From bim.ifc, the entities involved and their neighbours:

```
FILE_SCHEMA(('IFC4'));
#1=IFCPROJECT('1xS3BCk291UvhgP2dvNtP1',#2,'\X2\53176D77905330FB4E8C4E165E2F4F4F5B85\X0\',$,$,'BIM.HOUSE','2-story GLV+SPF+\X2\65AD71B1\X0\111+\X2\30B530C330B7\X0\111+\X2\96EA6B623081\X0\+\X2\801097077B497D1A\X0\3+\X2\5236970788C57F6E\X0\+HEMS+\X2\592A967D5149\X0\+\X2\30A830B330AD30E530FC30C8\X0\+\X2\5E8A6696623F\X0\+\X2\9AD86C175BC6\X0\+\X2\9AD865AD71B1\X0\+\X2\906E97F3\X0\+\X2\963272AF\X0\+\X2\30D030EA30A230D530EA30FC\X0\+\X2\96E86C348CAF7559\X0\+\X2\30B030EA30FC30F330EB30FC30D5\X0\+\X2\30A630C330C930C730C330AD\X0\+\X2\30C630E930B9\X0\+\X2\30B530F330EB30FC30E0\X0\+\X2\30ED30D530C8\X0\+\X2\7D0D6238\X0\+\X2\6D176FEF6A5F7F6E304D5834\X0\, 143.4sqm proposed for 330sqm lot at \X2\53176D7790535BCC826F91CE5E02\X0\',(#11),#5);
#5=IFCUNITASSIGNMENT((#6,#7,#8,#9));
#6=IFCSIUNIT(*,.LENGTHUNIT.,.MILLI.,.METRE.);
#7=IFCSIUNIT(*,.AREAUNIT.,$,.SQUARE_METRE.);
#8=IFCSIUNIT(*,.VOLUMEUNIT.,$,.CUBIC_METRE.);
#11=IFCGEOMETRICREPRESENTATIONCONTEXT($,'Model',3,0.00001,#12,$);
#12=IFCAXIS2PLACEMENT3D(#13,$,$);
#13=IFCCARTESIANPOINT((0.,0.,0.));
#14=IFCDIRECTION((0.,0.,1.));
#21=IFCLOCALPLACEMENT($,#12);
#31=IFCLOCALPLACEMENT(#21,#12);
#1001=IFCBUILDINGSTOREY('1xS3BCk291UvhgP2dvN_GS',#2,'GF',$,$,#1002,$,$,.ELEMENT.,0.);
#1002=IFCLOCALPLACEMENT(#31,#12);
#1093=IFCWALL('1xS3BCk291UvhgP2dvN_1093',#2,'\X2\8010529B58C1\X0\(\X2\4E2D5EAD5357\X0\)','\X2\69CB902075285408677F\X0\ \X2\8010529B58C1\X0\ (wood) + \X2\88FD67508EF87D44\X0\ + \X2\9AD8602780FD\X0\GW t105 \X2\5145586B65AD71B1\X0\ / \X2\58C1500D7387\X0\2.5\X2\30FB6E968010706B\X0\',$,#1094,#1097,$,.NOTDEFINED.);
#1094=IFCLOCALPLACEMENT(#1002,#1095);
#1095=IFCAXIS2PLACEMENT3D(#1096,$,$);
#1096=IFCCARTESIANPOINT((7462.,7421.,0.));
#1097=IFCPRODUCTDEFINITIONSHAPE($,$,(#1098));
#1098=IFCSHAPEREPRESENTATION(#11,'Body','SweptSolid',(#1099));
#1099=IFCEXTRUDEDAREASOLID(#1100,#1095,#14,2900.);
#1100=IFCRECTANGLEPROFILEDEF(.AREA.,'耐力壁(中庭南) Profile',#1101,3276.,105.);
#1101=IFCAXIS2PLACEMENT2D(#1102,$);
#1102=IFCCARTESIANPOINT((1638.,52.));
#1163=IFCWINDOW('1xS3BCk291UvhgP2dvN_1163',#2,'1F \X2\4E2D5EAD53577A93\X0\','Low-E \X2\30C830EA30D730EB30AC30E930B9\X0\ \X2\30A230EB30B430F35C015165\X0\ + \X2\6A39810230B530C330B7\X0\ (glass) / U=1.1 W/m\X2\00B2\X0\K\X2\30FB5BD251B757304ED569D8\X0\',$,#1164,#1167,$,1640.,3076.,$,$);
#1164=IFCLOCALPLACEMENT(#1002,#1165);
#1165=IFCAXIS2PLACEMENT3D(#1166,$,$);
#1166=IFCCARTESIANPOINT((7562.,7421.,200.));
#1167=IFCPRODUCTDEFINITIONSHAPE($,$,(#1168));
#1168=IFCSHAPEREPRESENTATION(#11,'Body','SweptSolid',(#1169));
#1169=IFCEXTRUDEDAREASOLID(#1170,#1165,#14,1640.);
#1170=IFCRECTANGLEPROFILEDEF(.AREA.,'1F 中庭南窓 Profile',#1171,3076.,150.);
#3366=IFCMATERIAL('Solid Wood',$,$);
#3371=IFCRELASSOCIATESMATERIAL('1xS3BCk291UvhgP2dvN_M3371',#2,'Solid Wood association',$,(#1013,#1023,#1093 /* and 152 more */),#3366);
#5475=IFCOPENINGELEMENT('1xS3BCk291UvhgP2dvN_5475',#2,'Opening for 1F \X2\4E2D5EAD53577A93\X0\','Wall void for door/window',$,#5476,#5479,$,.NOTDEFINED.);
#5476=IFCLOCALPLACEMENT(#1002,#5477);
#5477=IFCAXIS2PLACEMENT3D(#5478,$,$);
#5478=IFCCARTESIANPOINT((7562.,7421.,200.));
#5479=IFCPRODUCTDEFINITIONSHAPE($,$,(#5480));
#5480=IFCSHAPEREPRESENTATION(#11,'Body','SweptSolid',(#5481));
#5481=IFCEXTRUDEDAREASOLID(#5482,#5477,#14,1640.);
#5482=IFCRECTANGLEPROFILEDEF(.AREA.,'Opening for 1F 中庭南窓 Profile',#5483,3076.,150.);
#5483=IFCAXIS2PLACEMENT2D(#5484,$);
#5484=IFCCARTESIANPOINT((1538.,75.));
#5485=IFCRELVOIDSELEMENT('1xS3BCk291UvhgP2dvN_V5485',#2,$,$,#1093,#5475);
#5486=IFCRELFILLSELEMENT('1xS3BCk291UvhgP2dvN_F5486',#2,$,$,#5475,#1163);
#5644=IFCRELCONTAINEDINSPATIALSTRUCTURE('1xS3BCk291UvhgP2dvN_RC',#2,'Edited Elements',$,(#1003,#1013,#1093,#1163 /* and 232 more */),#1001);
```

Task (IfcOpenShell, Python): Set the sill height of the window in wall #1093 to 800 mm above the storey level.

```python
import numpy as np
import ifcopenshell
import ifcopenshell.api.geometry
import ifcopenshell.geom
import ifcopenshell.util.element
import ifcopenshell.util.placement
import ifcopenshell.util.shape
import ifcopenshell.util.unit

model = ifcopenshell.open("bim.ifc")
unit_scale = ifcopenshell.util.unit.calculate_unit_scale(model)

window = model.by_guid("1xS3BCk291UvhgP2dvN_1163")
opening = window.FillsVoids[0].RelatingOpeningElement
storey = ifcopenshell.util.element.get_container(window, ifc_class="IfcBuildingStorey")
level = ifcopenshell.util.placement.get_local_placement(storey.ObjectPlacement)[2, 3]

# The opening's origin need not be at the sill, so measure its lowest point.
shape = ifcopenshell.geom.create_shape(ifcopenshell.geom.settings(), opening)
bottom = ifcopenshell.util.shape.get_shape_bottom_elevation(shape, shape.geometry) / unit_scale
dz = level + 0.8 / unit_scale - bottom

shift = np.array([0.0, 0.0, dz])
# The window is not placed relative to its opening, so move both.
for product in (opening, window):
    matrix = ifcopenshell.util.placement.get_local_placement(product.ObjectPlacement)
    matrix[:3, 3] += shift
    ifcopenshell.api.geometry.edit_object_placement(model, product=product, matrix=matrix, is_si=False)

print(f"moved by {dz * unit_scale:+.3f} m")

model.write("bim_v2.ifc")
```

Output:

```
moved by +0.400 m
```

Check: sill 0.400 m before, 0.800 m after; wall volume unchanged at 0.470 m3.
